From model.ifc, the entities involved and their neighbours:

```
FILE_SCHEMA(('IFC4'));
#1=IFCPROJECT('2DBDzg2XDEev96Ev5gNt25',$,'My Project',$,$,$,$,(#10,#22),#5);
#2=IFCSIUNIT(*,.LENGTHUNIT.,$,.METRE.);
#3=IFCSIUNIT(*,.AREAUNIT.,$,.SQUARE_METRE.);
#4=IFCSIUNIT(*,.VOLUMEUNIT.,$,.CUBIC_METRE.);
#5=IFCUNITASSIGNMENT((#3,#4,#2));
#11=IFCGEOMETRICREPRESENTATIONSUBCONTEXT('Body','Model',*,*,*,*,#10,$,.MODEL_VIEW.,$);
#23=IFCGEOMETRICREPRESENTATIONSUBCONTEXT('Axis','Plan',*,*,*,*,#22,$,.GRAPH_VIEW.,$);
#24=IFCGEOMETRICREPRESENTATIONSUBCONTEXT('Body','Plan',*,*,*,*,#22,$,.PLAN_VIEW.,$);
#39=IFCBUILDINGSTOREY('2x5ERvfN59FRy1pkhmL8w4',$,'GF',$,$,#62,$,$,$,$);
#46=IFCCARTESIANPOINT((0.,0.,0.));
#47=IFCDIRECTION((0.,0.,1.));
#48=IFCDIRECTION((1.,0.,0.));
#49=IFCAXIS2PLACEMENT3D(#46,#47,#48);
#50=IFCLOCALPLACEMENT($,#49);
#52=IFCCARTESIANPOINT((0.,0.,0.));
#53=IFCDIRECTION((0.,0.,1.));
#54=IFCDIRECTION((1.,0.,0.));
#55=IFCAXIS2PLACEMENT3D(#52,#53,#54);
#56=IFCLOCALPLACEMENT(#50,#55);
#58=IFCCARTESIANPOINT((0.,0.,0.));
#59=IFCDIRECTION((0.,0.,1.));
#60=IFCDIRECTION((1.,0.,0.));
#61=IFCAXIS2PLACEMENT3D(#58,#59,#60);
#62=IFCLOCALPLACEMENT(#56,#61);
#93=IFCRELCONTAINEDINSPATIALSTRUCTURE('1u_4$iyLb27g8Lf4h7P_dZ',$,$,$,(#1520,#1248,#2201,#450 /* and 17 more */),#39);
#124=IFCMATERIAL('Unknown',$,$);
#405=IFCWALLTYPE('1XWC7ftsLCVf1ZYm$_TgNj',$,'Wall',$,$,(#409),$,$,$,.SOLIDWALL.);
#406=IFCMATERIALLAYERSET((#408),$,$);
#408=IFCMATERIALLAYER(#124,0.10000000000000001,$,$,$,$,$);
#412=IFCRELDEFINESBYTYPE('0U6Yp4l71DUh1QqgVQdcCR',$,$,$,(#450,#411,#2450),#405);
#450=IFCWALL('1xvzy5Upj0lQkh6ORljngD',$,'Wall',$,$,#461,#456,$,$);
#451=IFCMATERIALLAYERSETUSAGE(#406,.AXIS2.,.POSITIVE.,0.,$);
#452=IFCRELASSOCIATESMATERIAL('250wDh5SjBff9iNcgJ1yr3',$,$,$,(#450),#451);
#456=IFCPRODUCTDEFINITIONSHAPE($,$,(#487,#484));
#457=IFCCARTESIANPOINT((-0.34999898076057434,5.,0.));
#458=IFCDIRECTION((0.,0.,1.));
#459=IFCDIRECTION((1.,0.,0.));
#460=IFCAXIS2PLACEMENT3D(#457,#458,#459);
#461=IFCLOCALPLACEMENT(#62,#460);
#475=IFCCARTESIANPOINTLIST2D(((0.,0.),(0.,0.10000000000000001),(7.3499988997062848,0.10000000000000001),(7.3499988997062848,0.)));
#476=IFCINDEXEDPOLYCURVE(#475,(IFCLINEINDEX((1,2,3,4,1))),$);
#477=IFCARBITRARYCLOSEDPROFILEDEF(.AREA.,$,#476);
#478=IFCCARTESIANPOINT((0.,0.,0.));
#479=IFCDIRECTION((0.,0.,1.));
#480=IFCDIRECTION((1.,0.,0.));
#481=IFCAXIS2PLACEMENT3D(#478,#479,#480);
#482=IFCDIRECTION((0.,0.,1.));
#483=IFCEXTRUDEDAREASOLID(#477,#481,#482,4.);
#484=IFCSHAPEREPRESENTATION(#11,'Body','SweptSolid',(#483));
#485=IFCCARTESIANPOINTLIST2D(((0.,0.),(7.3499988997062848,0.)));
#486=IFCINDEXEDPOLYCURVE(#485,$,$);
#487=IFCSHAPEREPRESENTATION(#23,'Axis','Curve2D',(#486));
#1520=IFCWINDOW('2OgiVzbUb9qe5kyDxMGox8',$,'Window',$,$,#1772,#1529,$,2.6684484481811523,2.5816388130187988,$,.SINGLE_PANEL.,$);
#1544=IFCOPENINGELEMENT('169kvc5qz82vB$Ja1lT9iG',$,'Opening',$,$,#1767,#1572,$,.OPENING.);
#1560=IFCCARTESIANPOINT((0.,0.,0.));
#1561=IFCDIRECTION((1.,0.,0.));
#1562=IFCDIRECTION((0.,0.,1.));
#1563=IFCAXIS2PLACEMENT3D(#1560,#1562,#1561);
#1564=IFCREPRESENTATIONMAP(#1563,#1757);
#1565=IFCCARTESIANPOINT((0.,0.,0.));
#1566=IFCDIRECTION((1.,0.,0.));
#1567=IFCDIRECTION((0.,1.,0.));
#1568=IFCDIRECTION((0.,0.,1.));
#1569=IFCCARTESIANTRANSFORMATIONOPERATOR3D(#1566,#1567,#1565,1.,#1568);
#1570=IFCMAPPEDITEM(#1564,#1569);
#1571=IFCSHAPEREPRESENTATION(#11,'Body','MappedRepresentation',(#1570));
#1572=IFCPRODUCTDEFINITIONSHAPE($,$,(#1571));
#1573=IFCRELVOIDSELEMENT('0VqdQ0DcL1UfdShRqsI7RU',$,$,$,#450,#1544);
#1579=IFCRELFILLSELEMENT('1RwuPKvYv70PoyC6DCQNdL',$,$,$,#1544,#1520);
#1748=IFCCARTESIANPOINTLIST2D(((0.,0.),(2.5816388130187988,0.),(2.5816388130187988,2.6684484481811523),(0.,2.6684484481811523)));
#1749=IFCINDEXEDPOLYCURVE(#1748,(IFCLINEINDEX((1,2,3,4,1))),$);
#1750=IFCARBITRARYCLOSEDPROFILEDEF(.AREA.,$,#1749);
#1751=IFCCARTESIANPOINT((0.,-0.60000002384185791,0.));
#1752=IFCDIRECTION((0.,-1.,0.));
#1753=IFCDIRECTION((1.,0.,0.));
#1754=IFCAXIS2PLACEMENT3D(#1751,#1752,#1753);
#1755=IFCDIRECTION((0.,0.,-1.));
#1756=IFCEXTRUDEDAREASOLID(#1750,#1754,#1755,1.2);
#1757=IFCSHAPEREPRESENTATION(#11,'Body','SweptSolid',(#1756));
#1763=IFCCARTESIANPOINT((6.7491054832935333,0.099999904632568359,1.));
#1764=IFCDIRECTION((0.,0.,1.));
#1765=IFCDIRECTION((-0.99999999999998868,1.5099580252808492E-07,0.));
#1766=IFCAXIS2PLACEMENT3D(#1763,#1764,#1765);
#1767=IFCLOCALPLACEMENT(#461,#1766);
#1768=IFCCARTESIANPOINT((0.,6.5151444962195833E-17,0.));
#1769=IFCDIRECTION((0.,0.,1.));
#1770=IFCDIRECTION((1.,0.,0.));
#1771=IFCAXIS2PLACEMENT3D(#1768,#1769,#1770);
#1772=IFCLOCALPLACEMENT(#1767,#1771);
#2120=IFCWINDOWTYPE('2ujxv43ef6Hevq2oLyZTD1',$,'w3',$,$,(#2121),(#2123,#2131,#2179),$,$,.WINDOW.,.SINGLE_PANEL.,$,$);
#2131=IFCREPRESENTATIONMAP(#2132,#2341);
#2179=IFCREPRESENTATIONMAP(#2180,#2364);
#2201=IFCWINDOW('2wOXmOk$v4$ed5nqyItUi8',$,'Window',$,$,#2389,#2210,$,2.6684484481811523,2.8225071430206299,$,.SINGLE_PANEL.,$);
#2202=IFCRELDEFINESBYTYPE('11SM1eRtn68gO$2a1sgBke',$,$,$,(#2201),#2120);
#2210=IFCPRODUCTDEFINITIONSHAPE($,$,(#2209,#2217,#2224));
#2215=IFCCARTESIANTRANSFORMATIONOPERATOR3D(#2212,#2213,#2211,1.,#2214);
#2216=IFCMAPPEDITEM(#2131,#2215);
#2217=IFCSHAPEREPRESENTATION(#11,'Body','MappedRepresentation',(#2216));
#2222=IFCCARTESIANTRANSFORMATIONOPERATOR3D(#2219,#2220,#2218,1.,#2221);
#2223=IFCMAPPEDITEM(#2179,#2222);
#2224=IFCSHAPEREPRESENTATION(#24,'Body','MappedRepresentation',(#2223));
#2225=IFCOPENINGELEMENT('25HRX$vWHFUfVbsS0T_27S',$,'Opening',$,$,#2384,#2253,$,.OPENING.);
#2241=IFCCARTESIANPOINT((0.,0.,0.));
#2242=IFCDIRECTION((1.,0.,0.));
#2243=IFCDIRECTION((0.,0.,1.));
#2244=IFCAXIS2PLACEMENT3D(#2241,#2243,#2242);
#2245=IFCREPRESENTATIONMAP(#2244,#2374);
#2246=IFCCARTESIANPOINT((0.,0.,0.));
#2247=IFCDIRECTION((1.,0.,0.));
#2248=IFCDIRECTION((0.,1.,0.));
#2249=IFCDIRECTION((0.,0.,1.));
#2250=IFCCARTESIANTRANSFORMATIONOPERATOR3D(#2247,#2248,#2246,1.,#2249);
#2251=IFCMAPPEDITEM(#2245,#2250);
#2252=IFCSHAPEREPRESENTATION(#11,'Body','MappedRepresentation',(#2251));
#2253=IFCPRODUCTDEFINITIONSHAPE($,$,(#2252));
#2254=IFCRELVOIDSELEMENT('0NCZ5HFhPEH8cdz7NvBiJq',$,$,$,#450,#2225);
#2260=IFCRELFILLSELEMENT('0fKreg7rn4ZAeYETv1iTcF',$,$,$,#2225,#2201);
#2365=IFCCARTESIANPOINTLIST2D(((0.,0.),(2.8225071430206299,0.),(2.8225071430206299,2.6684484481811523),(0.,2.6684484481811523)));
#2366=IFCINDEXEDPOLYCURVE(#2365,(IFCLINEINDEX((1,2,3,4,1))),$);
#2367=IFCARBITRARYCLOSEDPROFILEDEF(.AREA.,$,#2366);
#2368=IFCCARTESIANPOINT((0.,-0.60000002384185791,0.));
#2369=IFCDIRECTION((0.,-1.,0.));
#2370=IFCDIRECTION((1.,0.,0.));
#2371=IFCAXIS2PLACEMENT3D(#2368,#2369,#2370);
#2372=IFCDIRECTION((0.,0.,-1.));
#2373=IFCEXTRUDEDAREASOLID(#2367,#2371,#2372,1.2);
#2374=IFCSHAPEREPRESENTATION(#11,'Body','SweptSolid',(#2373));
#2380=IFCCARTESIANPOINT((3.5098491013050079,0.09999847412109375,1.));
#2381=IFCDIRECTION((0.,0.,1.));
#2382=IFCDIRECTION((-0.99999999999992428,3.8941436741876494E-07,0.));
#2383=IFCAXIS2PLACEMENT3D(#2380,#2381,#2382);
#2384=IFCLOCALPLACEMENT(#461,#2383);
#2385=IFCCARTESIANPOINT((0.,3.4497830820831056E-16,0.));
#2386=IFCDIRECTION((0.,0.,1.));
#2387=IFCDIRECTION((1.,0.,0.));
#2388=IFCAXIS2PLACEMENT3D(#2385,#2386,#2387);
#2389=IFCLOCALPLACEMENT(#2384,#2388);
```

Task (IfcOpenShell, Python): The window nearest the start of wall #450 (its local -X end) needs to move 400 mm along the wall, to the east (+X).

```python
import ifcopenshell
import ifcopenshell.api.geometry
import ifcopenshell.util.placement
import ifcopenshell.util.unit

model = ifcopenshell.open("model.ifc")
unit_scale = ifcopenshell.util.unit.calculate_unit_scale(model)

window = model.by_id(2201)
opening = window.FillsVoids[0].RelatingOpeningElement
wall = opening.VoidsElements[0].RelatingBuildingElement

wall_matrix = ifcopenshell.util.placement.get_local_placement(wall.ObjectPlacement)
shift = wall_matrix[:3, 0] * 0.4 / unit_scale
before = ifcopenshell.util.placement.get_local_placement(window.ObjectPlacement)[:3, 3].copy()

# The window is placed relative to its opening, so it follows when the opening moves.
matrix = ifcopenshell.util.placement.get_local_placement(opening.ObjectPlacement)
matrix[:3, 3] += shift
ifcopenshell.api.geometry.edit_object_placement(
    model, product=opening, matrix=matrix, is_si=False, should_transform_children=True
)

after = ifcopenshell.util.placement.get_local_placement(window.ObjectPlacement)[:3, 3]
print("window moved by", (after - before).round(3) + 0.0)

model.write("model_edited.ifc")
```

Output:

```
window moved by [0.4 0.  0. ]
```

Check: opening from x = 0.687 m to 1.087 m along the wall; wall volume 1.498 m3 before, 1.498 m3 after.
